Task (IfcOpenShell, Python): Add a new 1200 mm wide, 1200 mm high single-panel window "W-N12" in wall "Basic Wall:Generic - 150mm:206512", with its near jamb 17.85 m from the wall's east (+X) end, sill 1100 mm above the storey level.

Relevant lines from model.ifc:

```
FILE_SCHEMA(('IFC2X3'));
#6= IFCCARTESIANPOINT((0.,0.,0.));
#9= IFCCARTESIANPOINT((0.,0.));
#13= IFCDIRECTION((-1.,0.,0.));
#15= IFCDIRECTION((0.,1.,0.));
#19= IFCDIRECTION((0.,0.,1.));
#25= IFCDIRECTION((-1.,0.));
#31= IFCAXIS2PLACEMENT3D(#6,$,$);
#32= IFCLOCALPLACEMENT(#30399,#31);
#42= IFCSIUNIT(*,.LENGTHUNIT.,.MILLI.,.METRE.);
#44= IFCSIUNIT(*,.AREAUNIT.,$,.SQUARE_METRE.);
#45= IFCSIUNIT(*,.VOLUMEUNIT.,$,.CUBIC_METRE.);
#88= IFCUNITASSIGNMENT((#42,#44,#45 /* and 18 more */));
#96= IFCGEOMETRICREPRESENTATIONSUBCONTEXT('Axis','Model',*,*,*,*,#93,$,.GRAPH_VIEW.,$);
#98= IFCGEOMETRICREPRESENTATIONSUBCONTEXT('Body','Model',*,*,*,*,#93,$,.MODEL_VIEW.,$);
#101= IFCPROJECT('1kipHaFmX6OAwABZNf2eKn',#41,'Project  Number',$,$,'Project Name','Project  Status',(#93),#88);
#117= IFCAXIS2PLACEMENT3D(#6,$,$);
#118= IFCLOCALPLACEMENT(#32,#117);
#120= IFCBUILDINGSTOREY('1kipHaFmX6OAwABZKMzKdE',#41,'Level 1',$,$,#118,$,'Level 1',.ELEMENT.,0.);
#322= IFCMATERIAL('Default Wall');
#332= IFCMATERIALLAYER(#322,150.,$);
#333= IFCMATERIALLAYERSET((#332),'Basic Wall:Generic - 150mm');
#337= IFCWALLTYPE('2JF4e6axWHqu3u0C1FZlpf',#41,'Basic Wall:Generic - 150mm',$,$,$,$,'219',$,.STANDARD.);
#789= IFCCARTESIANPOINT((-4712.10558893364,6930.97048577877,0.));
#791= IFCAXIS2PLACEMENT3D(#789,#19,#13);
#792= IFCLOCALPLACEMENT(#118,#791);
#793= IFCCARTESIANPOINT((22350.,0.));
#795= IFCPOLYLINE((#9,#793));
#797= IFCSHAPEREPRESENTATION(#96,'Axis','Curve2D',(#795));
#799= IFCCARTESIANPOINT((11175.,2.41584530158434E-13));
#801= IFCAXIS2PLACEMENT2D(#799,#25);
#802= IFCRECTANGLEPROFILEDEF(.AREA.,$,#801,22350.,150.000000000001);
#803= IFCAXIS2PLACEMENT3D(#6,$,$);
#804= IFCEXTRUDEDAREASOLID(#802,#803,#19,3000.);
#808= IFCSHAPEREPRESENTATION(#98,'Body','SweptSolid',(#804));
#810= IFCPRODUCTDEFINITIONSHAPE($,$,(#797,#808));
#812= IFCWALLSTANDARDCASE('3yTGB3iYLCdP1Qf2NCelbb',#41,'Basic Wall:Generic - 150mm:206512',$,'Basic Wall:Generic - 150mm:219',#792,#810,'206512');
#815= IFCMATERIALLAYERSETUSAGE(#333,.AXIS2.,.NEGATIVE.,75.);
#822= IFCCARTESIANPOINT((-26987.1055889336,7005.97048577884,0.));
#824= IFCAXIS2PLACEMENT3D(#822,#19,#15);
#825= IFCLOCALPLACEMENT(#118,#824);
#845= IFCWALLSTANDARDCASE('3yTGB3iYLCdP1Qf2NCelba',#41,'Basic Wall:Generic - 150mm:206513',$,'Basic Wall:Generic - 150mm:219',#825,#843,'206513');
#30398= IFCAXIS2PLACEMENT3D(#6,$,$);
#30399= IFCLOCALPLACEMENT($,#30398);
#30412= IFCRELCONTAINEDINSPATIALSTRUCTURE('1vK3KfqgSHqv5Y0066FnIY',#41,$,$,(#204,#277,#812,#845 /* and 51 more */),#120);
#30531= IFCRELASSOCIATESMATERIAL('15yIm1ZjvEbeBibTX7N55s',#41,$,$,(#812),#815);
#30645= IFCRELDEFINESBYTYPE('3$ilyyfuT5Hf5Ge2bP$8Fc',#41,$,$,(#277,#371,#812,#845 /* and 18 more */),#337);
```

```python
import numpy as np
import ifcopenshell
import ifcopenshell.api.feature
import ifcopenshell.api.geometry
import ifcopenshell.api.root
import ifcopenshell.api.spatial
import ifcopenshell.api.type
import ifcopenshell.geom
import ifcopenshell.util.element
import ifcopenshell.util.placement
import ifcopenshell.util.representation
import ifcopenshell.util.shape
import ifcopenshell.util.unit

model = ifcopenshell.open("model.ifc")
unit_scale = ifcopenshell.util.unit.calculate_unit_scale(model)
settings = ifcopenshell.geom.settings()


def volume(element):
    """Net volume in cubic metres, openings subtracted."""
    shape = ifcopenshell.geom.create_shape(settings, element)
    return ifcopenshell.util.shape.get_volume(shape.geometry)


wall = model.by_guid("3yTGB3iYLCdP1Qf2NCelbb")
storey = ifcopenshell.util.element.get_container(wall, ifc_class="IfcBuildingStorey")
context = ifcopenshell.util.representation.get_context(model, "Model", "Body", "MODEL_VIEW")
before = volume(wall)

width, height, from_end, sill = 1.2, 1.2, 17.85, 1.1  # metres

# The wall runs along its own X axis, and the end named is its -X end.
wall_shape = ifcopenshell.geom.create_shape(settings, wall)
x, y, z = ifcopenshell.util.shape.get_vertices(wall_shape.geometry).T
start = x.min() + from_end
face, thickness = float(y.min()), float(y.max() - y.min())
wall_matrix = ifcopenshell.util.placement.get_local_placement(wall.ObjectPlacement)
level = ifcopenshell.util.placement.get_local_placement(storey.ObjectPlacement)[2, 3]


def in_wall(x, y):
    """Placement at x, y metres in the wall's axes, at sill height."""
    matrix = wall_matrix.copy()
    matrix[:, 3] = wall_matrix @ np.array([x / unit_scale, y / unit_scale, 0.0, 1.0])
    matrix[2, 3] = level + sill / unit_scale
    return matrix


# Opening: a box that overshoots both wall faces by 50 mm.
opening = ifcopenshell.api.root.create_entity(model, ifc_class="IfcOpeningElement")
box = ifcopenshell.api.geometry.add_wall_representation(
    model, context=context, length=width, height=height, thickness=thickness + 0.1
)
ifcopenshell.api.geometry.assign_representation(model, product=opening, representation=box)
ifcopenshell.api.geometry.edit_object_placement(model, product=opening, matrix=in_wall(start, face - 0.05), is_si=False)
ifcopenshell.api.feature.add_feature(model, feature=opening, element=wall)

window = ifcopenshell.api.root.create_entity(model, ifc_class="IfcWindow", name="W-N12")
window.OverallWidth, window.OverallHeight = width / unit_scale, height / unit_scale
body = ifcopenshell.api.geometry.add_window_representation(
    model,
    context=context,
    overall_width=window.OverallWidth,
    overall_height=window.OverallHeight,
    partition_type="SINGLE_PANEL",
)
ifcopenshell.api.geometry.assign_representation(model, product=window, representation=body)
ifcopenshell.api.spatial.assign_container(model, products=[window], relating_structure=storey)
fills = ifcopenshell.api.feature.add_filling(model, opening=opening, element=window)
fills.OwnerHistory = window.OwnerHistory  # required in IFC2X3

# IFC2X3 keeps the operation on the window style.
style = ifcopenshell.api.root.create_entity(model, ifc_class="IfcWindowStyle", name="W-N12")
style.OperationType, style.ConstructionType = "SINGLE_PANEL", "NOTDEFINED"
style.ParameterTakesPrecedence = style.Sizeable = False
ifcopenshell.api.type.assign_type(model, related_objects=[window], relating_type=style)

# Centre the window in the wall's thickness.
ifcopenshell.api.geometry.edit_object_placement(model, product=window, matrix=in_wall(start, face), is_si=False)
window_shape = ifcopenshell.geom.create_shape(settings, window)
depth = ifcopenshell.util.shape.get_vertices(window_shape.geometry)[:, 1]
offset = face + thickness / 2 - (depth.min() + depth.max()) / 2
ifcopenshell.api.geometry.edit_object_placement(model, product=window, matrix=in_wall(start, offset), is_si=False)

after = volume(wall)

print(f"wall volume {before:.3f} -> {after:.3f} m3")

model.write("model_rev.ifc")
```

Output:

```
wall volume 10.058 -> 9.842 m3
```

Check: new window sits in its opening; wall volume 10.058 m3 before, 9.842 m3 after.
